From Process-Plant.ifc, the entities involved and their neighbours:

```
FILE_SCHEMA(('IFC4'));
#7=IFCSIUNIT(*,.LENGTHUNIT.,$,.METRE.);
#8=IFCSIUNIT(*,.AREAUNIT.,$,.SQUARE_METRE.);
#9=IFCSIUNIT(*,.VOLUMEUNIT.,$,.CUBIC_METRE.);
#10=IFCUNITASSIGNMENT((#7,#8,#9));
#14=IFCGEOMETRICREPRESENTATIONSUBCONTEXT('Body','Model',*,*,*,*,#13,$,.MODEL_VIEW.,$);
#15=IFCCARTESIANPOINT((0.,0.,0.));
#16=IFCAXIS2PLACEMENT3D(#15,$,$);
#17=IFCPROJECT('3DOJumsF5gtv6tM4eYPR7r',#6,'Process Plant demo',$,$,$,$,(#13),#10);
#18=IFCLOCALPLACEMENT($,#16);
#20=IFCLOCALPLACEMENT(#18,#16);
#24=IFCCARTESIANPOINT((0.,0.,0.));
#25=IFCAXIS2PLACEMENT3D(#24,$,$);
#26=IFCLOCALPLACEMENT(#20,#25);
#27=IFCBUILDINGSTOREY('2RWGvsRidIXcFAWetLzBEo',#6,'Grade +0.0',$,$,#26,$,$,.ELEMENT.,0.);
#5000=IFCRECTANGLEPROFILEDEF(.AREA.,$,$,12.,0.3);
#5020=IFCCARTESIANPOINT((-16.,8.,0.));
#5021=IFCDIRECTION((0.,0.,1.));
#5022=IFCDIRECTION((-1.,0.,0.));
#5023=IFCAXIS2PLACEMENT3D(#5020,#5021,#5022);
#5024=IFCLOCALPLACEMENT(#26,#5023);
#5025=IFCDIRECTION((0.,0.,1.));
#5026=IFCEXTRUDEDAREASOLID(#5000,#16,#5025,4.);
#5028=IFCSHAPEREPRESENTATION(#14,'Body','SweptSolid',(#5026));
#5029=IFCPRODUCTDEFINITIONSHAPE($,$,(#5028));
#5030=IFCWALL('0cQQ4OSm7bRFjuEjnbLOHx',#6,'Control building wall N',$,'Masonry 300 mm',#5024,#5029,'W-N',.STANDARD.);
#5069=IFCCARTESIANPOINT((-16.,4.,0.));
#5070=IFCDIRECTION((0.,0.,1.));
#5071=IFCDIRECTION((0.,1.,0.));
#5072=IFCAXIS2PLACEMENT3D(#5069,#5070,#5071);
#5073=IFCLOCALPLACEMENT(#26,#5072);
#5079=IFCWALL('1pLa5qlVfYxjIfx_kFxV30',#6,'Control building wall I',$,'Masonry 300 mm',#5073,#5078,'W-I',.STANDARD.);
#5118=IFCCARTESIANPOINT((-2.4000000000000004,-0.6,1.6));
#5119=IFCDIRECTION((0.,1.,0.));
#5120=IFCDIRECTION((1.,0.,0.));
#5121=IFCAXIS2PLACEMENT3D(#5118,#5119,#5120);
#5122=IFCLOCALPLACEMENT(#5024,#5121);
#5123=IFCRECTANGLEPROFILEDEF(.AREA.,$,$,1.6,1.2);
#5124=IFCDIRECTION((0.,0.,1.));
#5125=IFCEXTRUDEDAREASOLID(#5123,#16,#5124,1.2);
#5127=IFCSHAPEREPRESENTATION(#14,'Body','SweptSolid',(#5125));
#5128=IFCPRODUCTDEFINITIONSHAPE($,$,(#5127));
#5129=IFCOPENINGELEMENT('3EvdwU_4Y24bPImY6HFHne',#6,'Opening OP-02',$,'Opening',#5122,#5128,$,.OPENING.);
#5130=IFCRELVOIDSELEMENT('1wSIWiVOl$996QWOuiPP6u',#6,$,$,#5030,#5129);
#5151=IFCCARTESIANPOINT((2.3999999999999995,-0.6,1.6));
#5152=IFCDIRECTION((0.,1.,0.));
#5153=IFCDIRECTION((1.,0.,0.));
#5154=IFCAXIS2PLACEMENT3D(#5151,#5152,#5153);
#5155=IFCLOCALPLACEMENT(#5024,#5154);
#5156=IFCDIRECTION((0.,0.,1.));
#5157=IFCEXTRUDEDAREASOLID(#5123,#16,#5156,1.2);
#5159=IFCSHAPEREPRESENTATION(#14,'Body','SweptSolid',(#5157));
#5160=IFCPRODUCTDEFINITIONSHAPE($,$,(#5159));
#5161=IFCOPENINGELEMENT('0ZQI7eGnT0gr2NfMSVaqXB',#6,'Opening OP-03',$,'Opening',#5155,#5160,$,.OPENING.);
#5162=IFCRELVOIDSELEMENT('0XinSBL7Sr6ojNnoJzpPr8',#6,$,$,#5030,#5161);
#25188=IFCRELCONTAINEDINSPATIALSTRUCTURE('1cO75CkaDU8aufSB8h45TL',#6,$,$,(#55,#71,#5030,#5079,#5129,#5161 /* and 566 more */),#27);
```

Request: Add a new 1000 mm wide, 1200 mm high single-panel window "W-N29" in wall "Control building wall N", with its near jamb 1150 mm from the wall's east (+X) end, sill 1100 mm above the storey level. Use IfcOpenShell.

```python
import numpy as np
import ifcopenshell
import ifcopenshell.api.feature
import ifcopenshell.api.geometry
import ifcopenshell.api.root
import ifcopenshell.api.spatial
import ifcopenshell.geom
import ifcopenshell.util.element
import ifcopenshell.util.placement
import ifcopenshell.util.representation
import ifcopenshell.util.shape
import ifcopenshell.util.unit

model = ifcopenshell.open("Process-Plant.ifc")
unit_scale = ifcopenshell.util.unit.calculate_unit_scale(model)
settings = ifcopenshell.geom.settings()


def volume(element):
    """Net volume in cubic metres, openings subtracted."""
    shape = ifcopenshell.geom.create_shape(settings, element)
    return ifcopenshell.util.shape.get_volume(shape.geometry)


wall = model.by_id(5030)
storey = ifcopenshell.util.element.get_container(wall, ifc_class="IfcBuildingStorey")
context = ifcopenshell.util.representation.get_context(model, "Model", "Body", "MODEL_VIEW")
before = volume(wall)

width, height, from_end, sill = 1, 1.2, 1.15, 1.1  # metres

# The wall runs along its own X axis, and the end named is its -X end.
wall_shape = ifcopenshell.geom.create_shape(settings, wall)
x, y, z = ifcopenshell.util.shape.get_vertices(wall_shape.geometry).T
start = x.min() + from_end
face, thickness = float(y.min()), float(y.max() - y.min())
wall_matrix = ifcopenshell.util.placement.get_local_placement(wall.ObjectPlacement)
level = ifcopenshell.util.placement.get_local_placement(storey.ObjectPlacement)[2, 3]


def in_wall(x, y):
    """Placement at x, y metres in the wall's axes, at sill height."""
    matrix = wall_matrix.copy()
    matrix[:, 3] = wall_matrix @ np.array([x / unit_scale, y / unit_scale, 0.0, 1.0])
    matrix[2, 3] = level + sill / unit_scale
    return matrix


# Opening: a box that overshoots both wall faces by 50 mm.
opening = ifcopenshell.api.root.create_entity(model, ifc_class="IfcOpeningElement", predefined_type="OPENING")
box = ifcopenshell.api.geometry.add_wall_representation(
    model, context=context, length=width, height=height, thickness=thickness + 0.1
)
ifcopenshell.api.geometry.assign_representation(model, product=opening, representation=box)
ifcopenshell.api.geometry.edit_object_placement(model, product=opening, matrix=in_wall(start, face - 0.05), is_si=False)
ifcopenshell.api.feature.add_feature(model, feature=opening, element=wall)

window = ifcopenshell.api.root.create_entity(model, ifc_class="IfcWindow", name="W-N29", predefined_type="WINDOW")
window.OverallWidth, window.OverallHeight = width / unit_scale, height / unit_scale
window.PartitioningType = "SINGLE_PANEL"
body = ifcopenshell.api.geometry.add_window_representation(
    model,
    context=context,
    overall_width=window.OverallWidth,
    overall_height=window.OverallHeight,
    partition_type="SINGLE_PANEL",
)
ifcopenshell.api.geometry.assign_representation(model, product=window, representation=body)
ifcopenshell.api.spatial.assign_container(model, products=[window], relating_structure=storey)
ifcopenshell.api.feature.add_filling(model, opening=opening, element=window)

# Centre the window in the wall's thickness.
ifcopenshell.api.geometry.edit_object_placement(model, product=window, matrix=in_wall(start, face), is_si=False)
window_shape = ifcopenshell.geom.create_shape(settings, window)
depth = ifcopenshell.util.shape.get_vertices(window_shape.geometry)[:, 1]
offset = face + thickness / 2 - (depth.min() + depth.max()) / 2
ifcopenshell.api.geometry.edit_object_placement(model, product=window, matrix=in_wall(start, offset), is_si=False)

after = volume(wall)

print(f"wall volume {before:.3f} -> {after:.3f} m3")

model.write("Process-Plant_v2.ifc")
```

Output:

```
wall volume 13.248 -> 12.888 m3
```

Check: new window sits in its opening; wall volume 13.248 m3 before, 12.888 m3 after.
